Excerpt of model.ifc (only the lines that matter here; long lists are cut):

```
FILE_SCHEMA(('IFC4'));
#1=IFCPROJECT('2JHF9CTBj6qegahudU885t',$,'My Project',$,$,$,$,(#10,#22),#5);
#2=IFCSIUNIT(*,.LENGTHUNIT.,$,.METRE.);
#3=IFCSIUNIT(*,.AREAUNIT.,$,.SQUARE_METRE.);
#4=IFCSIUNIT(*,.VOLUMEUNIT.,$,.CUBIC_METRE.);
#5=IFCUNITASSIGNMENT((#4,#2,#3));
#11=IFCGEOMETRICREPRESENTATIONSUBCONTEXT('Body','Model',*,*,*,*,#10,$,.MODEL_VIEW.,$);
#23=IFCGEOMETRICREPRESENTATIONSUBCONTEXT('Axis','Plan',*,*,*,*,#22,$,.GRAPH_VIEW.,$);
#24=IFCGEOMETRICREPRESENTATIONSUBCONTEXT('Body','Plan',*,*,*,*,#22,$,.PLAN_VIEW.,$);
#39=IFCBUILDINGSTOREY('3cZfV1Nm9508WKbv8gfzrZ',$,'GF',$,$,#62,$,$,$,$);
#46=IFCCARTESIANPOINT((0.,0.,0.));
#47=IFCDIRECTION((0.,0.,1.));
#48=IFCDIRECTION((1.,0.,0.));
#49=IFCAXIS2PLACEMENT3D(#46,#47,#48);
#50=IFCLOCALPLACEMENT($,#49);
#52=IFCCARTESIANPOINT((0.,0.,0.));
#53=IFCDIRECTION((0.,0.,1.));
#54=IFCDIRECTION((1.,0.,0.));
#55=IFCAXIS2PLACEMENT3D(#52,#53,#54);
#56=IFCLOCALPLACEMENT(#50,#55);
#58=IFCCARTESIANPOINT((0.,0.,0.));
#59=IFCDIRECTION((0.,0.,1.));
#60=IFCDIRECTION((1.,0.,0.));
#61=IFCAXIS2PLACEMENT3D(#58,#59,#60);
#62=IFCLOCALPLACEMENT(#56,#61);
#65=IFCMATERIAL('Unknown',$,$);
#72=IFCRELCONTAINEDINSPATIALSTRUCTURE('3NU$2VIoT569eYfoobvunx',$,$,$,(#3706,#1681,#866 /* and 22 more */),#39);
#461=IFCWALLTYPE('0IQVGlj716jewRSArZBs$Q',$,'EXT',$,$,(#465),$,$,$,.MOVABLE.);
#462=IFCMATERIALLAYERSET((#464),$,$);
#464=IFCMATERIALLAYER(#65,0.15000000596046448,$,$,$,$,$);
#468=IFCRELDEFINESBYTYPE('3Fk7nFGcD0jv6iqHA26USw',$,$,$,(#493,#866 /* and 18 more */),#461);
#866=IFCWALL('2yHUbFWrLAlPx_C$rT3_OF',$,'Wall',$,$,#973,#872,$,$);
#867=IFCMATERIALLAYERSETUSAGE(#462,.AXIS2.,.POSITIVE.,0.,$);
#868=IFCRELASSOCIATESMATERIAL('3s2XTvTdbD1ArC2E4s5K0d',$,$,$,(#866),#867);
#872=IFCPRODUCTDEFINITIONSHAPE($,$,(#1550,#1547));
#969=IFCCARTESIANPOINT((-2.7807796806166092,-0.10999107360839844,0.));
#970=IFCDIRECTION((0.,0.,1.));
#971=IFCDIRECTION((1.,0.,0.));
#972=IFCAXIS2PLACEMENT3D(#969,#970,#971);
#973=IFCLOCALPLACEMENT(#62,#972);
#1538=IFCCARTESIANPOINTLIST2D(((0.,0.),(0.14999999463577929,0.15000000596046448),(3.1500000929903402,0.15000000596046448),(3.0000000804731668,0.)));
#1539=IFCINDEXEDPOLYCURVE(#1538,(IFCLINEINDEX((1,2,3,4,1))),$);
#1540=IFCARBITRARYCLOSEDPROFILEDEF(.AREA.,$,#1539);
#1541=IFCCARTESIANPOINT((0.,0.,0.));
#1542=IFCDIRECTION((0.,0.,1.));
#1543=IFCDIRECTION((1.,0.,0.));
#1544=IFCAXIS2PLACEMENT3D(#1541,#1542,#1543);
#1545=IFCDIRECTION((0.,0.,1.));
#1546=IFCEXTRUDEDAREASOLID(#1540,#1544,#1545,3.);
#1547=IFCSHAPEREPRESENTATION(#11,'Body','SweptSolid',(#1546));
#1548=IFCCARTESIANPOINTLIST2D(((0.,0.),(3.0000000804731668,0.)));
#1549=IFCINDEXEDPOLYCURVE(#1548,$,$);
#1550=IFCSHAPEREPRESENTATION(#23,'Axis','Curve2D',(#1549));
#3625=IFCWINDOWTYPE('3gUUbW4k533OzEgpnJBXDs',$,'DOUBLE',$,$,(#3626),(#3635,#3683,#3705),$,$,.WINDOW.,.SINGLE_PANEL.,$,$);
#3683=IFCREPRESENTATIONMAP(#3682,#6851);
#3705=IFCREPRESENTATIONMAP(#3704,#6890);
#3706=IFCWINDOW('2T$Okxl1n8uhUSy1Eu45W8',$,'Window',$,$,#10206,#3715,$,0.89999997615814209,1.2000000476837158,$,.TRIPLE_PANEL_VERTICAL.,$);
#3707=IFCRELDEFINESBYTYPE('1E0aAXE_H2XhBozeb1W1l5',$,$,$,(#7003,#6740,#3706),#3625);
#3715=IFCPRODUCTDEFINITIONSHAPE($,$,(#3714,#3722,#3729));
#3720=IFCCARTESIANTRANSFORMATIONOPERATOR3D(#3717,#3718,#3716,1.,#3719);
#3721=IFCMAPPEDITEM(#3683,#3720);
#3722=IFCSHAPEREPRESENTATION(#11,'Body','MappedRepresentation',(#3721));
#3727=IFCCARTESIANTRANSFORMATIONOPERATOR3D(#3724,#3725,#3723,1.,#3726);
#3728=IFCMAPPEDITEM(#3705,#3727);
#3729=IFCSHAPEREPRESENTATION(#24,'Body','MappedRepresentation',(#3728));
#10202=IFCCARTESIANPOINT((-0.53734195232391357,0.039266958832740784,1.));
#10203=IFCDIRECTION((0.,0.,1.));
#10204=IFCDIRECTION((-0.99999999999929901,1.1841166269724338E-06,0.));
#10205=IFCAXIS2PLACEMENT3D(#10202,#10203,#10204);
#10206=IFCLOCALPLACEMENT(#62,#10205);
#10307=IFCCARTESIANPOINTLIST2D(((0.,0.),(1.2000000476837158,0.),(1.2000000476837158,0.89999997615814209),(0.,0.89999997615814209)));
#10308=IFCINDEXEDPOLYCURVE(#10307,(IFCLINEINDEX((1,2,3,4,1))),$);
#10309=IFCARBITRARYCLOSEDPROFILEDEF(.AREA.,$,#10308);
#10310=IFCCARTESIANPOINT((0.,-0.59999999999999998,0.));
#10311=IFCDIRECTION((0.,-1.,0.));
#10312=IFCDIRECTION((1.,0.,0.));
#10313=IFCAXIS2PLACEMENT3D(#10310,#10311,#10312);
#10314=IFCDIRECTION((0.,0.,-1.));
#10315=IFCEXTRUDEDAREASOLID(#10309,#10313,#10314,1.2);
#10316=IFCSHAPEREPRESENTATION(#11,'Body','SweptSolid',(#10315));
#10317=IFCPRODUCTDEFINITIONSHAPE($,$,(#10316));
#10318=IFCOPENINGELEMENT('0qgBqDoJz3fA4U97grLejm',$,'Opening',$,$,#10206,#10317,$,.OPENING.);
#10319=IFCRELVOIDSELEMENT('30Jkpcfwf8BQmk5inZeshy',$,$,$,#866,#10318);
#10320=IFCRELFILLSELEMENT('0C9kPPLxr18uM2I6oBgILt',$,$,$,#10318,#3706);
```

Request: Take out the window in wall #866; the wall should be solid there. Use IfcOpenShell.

```python
import ifcopenshell
import ifcopenshell.api.feature
import ifcopenshell.api.root
import ifcopenshell.geom
import ifcopenshell.util.shape

model = ifcopenshell.open("model.ifc")
settings = ifcopenshell.geom.settings()


def volume(element):
    """Net volume in cubic metres, openings subtracted."""
    shape = ifcopenshell.geom.create_shape(settings, element)
    return ifcopenshell.util.shape.get_volume(shape.geometry)


window = model.by_id(3706)
opening = window.FillsVoids[0].RelatingOpeningElement
wall = opening.VoidsElements[0].RelatingBuildingElement
before = volume(wall)

ifcopenshell.api.root.remove_product(model, product=window)
ifcopenshell.api.feature.remove_feature(model, feature=opening)

after = volume(wall)

print(f"wall volume {before:.3f} -> {after:.3f} m3")

model.write("model-out.ifc")
```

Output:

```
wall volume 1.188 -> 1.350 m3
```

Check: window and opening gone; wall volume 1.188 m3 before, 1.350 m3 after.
